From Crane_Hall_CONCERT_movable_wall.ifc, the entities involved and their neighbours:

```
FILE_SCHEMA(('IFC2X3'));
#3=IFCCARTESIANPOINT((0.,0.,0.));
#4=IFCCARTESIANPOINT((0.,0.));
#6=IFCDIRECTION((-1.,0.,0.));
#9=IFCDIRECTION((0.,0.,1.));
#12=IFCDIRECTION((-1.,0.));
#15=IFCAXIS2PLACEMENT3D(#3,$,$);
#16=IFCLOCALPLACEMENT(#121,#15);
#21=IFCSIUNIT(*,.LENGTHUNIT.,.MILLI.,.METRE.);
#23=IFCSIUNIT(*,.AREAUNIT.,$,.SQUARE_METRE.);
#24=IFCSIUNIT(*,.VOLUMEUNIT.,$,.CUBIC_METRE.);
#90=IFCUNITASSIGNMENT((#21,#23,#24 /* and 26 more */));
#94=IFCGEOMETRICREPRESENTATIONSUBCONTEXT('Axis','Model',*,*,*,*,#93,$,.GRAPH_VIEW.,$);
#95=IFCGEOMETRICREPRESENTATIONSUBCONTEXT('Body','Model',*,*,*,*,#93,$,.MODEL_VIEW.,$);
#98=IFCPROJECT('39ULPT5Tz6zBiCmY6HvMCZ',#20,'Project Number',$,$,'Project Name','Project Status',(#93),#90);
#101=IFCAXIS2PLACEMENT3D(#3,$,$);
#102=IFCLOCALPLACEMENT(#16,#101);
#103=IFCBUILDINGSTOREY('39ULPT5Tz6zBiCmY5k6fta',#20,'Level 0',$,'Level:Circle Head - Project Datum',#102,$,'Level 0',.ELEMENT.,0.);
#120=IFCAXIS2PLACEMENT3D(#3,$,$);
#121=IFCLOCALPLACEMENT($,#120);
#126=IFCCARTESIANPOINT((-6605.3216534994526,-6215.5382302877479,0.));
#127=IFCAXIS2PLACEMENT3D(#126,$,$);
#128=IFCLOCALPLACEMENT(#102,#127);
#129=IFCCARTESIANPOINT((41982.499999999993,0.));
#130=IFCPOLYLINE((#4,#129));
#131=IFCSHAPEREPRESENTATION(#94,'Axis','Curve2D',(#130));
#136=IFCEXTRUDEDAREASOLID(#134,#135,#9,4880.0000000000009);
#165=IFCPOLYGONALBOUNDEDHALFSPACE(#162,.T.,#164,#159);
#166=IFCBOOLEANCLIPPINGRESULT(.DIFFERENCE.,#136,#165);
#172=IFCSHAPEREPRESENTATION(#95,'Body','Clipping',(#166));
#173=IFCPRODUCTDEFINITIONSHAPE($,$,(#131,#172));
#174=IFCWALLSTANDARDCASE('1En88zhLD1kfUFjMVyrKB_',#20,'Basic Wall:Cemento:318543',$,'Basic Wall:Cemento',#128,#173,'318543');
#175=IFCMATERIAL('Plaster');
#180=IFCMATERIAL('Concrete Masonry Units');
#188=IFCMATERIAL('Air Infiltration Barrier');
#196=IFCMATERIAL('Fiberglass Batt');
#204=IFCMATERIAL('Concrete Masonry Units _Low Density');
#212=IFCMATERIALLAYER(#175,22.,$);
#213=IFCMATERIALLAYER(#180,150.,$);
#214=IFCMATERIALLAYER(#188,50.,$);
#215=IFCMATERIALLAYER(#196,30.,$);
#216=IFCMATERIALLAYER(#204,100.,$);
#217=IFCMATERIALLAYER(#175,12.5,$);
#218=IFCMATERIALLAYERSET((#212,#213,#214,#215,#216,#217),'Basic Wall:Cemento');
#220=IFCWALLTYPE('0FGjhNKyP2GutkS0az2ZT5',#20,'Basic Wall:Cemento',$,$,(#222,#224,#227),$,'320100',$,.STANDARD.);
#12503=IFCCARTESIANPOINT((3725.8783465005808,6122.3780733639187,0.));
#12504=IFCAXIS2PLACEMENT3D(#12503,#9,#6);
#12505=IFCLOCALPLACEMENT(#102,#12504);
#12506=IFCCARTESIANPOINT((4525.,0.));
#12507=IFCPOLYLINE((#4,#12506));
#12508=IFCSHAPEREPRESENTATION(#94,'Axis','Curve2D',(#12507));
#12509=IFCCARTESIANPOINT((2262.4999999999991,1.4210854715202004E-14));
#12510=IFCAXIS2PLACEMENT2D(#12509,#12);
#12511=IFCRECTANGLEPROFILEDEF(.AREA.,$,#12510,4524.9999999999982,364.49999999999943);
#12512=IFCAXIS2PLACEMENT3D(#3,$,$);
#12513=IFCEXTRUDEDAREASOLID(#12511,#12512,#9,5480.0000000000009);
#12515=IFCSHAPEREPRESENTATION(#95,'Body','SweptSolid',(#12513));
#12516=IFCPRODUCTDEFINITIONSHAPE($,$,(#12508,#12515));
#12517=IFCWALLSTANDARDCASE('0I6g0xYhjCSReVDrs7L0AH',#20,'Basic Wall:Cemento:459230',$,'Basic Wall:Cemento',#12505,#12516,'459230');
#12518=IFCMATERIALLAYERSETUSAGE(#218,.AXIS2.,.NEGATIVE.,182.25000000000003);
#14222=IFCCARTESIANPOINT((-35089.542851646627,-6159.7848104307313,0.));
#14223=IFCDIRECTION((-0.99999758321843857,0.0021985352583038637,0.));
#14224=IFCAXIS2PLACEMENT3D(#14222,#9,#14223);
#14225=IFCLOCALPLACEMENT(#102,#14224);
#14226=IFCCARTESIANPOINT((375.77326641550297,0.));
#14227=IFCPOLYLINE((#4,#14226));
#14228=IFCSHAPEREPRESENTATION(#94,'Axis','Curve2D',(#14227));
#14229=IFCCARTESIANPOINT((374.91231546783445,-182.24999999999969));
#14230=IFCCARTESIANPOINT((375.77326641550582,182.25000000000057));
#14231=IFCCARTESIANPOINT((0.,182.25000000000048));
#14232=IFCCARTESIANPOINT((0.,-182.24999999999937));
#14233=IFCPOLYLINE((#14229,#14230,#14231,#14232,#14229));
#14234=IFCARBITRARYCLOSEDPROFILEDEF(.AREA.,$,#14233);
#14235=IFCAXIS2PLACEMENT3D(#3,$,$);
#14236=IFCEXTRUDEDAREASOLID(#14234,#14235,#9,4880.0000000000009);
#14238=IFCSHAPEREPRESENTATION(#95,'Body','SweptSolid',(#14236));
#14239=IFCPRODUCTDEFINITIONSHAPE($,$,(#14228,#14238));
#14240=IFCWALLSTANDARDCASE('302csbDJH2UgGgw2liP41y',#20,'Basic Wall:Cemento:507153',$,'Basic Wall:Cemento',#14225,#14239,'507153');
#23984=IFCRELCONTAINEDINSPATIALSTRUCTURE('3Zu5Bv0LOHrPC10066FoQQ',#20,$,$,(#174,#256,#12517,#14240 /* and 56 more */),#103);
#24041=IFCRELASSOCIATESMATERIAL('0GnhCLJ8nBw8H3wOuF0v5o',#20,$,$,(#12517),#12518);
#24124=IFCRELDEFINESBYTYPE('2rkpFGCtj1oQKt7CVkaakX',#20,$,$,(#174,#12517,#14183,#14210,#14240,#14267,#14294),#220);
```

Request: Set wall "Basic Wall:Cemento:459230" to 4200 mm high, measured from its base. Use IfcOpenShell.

```python
import ifcopenshell
import ifcopenshell.geom
import ifcopenshell.util.representation
import ifcopenshell.util.shape
import ifcopenshell.util.unit

model = ifcopenshell.open("Crane_Hall_CONCERT_movable_wall.ifc")
unit_scale = ifcopenshell.util.unit.calculate_unit_scale(model)
settings = ifcopenshell.geom.settings()


def volume(element):
    """Net volume in cubic metres, openings subtracted."""
    shape = ifcopenshell.geom.create_shape(settings, element)
    return ifcopenshell.util.shape.get_volume(shape.geometry)


wall = model.by_guid("0I6g0xYhjCSReVDrs7L0AH")
before = volume(wall)

body = ifcopenshell.util.representation.get_representation(wall, "Model", "Body")
solid = body.Items[0]
old_height = solid.Depth
solid.Depth = 4.2 / unit_scale
after = volume(wall)

print(f"height {old_height:g} -> {solid.Depth:g}, volume {before:.3f} -> {after:.3f} m3")

model.write("Crane_Hall_CONCERT_movable_wall_updated.ifc")
```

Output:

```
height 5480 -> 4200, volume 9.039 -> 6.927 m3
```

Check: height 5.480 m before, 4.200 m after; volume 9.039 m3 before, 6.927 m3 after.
